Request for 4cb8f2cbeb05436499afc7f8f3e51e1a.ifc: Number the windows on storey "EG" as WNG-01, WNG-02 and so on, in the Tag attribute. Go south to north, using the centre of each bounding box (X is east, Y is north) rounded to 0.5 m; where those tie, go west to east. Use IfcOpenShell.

First a look at what the model holds.

```python
import ifcopenshell
import ifcopenshell.util.element
import ifcopenshell.util.placement

model = ifcopenshell.open("4cb8f2cbeb05436499afc7f8f3e51e1a.ifc")
print(model.schema)
storey = next(s for s in model.by_type("IfcBuildingStorey") if s.Name == "EG")
windows = [e for e in ifcopenshell.util.element.get_decomposition(storey) if e.is_a("IfcWindow")]
for e in sorted(windows, key=lambda e: e.id()):
    origin = ifcopenshell.util.placement.get_local_placement(e.ObjectPlacement)[:3, 3]
    print(e.id(), e.Tag, e.Name, origin.round(2) + 0.0, sep=" | ")
```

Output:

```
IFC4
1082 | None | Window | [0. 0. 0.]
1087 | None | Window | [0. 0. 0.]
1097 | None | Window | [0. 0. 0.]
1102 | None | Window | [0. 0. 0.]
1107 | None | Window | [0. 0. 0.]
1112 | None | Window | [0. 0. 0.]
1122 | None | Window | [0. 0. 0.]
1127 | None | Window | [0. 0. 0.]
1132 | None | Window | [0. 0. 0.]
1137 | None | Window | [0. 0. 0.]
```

```python
import ifcopenshell
import ifcopenshell.geom
import ifcopenshell.util.element
import ifcopenshell.util.shape

model = ifcopenshell.open("4cb8f2cbeb05436499afc7f8f3e51e1a.ifc")
settings = ifcopenshell.geom.settings()
settings.set("use-world-coords", True)


def centre(element):
    shape = ifcopenshell.geom.create_shape(settings, element)
    return ifcopenshell.util.shape.get_bbox_centroid(shape.geometry)


storey = next(s for s in model.by_type("IfcBuildingStorey") if s.Name == "EG")
windows = [e for e in ifcopenshell.util.element.get_decomposition(storey) if e.is_a("IfcWindow")]

# Insertion points can sit at a corner or the storey origin, so sort by the geometry (in metres).
centres = {e: centre(e) for e in windows}
windows.sort(key=lambda e: (round(centres[e][1] / 0.5), centres[e][0]))

for i, e in enumerate(windows, start=1):
    number = f"WNG-{i:02d}"
    e.Tag = number
    print(e.id(), number)

model.write("4cb8f2cbeb05436499afc7f8f3e51e1a_v2.ifc")
```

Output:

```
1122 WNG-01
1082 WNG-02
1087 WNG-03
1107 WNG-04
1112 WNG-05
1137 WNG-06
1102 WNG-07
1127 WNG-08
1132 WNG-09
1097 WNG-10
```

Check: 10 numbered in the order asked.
